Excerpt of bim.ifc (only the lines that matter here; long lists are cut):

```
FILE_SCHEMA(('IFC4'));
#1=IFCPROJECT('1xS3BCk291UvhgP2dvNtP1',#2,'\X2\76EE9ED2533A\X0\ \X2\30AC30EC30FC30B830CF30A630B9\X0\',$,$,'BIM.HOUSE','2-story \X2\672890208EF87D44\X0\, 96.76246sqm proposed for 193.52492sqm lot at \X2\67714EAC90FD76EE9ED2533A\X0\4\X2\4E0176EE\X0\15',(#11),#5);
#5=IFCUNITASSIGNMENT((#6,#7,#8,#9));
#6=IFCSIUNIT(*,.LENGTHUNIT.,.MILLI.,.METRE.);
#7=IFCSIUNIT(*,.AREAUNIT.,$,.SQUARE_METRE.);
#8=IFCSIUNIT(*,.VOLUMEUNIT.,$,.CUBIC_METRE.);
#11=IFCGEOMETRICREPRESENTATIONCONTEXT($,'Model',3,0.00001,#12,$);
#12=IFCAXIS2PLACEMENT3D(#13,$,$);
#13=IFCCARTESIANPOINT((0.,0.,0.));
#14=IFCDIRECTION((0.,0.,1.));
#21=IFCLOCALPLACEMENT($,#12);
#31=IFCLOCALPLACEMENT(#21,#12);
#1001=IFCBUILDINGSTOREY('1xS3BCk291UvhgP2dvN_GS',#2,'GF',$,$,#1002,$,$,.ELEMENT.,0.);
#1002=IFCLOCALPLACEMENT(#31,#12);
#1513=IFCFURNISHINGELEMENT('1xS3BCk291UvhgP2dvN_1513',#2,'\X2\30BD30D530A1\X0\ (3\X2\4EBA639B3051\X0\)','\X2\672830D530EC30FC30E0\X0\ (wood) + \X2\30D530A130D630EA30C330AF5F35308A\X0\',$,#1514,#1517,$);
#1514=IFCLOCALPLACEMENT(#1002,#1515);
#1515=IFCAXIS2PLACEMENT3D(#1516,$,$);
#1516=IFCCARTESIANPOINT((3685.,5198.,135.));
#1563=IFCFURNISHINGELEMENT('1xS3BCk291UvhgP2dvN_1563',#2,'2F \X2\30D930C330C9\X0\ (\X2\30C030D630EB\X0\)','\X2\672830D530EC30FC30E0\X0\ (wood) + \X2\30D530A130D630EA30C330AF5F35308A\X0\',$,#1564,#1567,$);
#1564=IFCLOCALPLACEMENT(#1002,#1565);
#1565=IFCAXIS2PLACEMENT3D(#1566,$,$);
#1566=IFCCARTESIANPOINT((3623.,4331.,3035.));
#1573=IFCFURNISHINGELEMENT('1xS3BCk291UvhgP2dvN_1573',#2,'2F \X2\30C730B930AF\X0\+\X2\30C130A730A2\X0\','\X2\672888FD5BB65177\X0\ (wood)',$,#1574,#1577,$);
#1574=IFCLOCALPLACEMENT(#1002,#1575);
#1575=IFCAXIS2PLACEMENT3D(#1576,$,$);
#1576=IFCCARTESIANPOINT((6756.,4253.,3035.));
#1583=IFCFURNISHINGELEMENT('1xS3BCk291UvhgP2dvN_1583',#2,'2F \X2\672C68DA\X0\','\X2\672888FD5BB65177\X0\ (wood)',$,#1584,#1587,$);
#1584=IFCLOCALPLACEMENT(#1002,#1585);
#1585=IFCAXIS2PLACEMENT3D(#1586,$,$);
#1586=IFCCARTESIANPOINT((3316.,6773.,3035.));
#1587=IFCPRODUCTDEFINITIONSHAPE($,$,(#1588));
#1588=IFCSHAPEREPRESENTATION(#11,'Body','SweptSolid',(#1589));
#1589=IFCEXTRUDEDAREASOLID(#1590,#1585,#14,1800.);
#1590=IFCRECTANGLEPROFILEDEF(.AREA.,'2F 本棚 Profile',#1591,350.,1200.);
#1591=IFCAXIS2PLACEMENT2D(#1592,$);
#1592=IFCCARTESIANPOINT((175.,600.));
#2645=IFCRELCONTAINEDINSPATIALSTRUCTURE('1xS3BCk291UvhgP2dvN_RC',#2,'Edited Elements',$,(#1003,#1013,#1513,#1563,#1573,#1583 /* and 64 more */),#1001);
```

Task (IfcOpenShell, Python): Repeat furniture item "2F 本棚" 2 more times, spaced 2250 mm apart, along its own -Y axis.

```python
import ifcopenshell
import ifcopenshell.api.geometry
import ifcopenshell.api.root
import ifcopenshell.util.element
import ifcopenshell.util.placement
import ifcopenshell.util.unit

model = ifcopenshell.open("bim.ifc")
unit_scale = ifcopenshell.util.unit.calculate_unit_scale(model)


def reuse_history(source, copy):
    """copy_class also copies each property set's owner history, people and application; keep the originals."""
    for rel in copy.IsDefinedBy:
        if rel.is_a("IfcRelDefinesByProperties") and (history := rel.RelatingPropertyDefinition.OwnerHistory):
            rel.RelatingPropertyDefinition.OwnerHistory = source.OwnerHistory
            ifcopenshell.util.element.remove_deep2(model, history)


source = model.by_id(1583)
base = ifcopenshell.util.placement.get_local_placement(source.ObjectPlacement)
step = -base[:3, 1] * 2.25 / unit_scale

for i in range(1, 3):
    copy = ifcopenshell.api.root.copy_class(model, product=source)
    copy.Representation = ifcopenshell.util.element.copy_deep(
        model, source.Representation, exclude=["IfcGeometricRepresentationContext", "IfcRepresentationMap"]
    )
    reuse_history(source, copy)
    matrix = base.copy()
    matrix[:3, 3] += i * step
    print("added at", matrix[:3, 3].round(3) + 0.0)
    ifcopenshell.api.geometry.edit_object_placement(model, product=copy, matrix=matrix, is_si=False)

model.write("bim_rev.ifc")
```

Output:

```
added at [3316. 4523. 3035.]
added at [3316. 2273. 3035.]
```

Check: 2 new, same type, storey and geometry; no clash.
